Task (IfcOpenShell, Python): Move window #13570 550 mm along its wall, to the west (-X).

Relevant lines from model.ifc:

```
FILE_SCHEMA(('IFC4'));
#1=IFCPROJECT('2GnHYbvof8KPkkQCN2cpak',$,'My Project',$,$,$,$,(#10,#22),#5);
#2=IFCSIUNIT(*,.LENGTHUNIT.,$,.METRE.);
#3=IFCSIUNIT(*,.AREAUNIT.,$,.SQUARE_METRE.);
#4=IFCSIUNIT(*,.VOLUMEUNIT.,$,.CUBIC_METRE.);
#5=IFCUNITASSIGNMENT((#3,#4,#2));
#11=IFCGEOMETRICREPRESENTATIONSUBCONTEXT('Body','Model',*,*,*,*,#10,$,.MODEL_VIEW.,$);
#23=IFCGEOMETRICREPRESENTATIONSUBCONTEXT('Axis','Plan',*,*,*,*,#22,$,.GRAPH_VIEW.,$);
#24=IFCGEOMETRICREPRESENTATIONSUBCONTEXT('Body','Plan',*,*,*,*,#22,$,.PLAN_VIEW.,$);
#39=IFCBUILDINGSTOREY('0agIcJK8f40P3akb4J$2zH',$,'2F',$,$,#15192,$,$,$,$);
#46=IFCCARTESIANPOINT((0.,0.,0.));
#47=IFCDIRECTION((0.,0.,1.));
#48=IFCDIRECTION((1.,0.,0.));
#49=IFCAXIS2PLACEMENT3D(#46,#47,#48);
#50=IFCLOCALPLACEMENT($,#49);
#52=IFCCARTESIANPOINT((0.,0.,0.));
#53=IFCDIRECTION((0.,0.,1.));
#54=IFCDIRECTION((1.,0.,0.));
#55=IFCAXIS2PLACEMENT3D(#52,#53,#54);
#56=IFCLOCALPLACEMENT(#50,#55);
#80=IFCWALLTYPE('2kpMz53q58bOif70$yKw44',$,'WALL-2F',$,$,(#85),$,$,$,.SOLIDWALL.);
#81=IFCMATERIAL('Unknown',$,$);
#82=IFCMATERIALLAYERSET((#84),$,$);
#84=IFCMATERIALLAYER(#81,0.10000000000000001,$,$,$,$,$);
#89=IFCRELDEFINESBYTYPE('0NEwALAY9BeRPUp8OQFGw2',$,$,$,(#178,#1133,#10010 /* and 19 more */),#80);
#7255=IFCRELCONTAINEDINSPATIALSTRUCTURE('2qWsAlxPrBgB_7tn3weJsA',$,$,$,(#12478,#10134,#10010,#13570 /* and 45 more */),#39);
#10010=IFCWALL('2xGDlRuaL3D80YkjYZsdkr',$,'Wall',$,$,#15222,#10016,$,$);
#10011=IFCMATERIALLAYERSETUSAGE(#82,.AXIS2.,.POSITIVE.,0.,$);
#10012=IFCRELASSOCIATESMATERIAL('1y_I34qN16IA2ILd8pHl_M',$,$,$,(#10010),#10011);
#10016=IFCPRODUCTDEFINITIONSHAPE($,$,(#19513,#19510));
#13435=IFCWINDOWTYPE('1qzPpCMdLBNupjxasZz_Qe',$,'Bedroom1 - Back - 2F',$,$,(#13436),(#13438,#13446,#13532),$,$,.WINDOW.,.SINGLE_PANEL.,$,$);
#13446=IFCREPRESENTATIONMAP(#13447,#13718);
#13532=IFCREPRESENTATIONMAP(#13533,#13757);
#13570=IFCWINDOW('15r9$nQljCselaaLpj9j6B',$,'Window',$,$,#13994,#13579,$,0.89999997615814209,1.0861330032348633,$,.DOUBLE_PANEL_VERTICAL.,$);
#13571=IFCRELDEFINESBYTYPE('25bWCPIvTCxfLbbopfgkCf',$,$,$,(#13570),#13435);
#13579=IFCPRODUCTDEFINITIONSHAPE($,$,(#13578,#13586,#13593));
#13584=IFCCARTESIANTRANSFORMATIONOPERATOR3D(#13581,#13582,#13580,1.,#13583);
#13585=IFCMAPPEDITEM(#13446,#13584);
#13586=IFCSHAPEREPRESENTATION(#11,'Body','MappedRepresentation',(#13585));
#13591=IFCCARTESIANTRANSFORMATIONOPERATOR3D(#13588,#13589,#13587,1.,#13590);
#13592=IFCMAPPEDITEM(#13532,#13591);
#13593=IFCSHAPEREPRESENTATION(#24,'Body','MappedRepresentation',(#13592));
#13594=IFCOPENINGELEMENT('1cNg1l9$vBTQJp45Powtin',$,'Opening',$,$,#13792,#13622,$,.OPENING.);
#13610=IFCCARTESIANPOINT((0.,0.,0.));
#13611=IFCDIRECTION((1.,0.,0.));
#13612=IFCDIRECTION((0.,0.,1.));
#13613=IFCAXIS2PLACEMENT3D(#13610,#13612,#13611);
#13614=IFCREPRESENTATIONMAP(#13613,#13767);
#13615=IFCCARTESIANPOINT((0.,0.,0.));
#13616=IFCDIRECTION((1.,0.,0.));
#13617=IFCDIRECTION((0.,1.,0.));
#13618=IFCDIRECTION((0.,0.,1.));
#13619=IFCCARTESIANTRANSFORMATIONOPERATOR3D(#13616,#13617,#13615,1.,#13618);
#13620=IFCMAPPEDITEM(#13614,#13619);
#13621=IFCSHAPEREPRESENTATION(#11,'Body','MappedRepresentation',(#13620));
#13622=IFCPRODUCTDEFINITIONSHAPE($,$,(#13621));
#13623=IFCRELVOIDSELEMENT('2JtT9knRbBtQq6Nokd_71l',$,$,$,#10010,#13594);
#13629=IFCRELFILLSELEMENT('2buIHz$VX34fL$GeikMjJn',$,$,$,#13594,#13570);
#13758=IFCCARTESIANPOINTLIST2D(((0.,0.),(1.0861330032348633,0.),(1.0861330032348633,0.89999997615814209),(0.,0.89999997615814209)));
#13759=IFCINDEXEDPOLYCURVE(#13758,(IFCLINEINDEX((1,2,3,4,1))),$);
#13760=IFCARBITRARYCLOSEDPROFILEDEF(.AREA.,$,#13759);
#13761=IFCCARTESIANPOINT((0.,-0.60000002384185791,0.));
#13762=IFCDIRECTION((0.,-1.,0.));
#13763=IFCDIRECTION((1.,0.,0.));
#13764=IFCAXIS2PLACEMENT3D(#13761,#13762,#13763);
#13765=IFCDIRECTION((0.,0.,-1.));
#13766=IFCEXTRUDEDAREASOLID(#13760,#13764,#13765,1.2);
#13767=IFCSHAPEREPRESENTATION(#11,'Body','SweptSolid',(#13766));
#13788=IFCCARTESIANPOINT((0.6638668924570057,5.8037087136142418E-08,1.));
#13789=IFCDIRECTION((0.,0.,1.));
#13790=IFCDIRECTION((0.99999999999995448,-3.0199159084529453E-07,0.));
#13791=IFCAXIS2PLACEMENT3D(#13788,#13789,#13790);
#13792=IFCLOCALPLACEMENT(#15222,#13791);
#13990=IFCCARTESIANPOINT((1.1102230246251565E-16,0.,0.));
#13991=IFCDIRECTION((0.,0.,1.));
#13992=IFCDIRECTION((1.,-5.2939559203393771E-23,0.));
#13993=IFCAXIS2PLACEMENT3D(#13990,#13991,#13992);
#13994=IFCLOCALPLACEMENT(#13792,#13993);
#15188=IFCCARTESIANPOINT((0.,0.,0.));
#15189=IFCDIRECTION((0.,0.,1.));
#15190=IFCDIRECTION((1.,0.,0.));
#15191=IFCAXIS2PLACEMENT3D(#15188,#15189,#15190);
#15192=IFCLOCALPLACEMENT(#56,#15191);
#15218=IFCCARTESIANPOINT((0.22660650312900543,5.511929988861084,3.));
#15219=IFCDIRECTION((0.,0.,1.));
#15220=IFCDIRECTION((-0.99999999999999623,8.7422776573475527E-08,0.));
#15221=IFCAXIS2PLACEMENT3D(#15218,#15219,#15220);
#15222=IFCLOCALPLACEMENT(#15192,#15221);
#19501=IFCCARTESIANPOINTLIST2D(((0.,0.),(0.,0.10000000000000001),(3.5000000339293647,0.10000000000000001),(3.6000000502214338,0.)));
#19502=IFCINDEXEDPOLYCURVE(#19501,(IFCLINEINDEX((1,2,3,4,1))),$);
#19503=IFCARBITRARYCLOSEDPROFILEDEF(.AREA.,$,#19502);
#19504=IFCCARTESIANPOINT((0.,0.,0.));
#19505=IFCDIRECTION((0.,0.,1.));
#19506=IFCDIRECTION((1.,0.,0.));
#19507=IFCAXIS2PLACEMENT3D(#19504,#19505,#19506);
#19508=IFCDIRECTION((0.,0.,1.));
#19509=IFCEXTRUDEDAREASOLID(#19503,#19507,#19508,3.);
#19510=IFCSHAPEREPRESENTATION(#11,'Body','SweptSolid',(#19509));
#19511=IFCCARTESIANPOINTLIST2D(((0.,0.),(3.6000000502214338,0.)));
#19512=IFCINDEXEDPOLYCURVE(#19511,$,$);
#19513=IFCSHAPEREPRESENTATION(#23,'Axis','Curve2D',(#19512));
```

```python
import ifcopenshell
import ifcopenshell.api.geometry
import ifcopenshell.util.placement
import ifcopenshell.util.unit

model = ifcopenshell.open("model.ifc")
unit_scale = ifcopenshell.util.unit.calculate_unit_scale(model)

window = model.by_guid("15r9$nQljCselaaLpj9j6B")
opening = window.FillsVoids[0].RelatingOpeningElement
wall = opening.VoidsElements[0].RelatingBuildingElement

wall_matrix = ifcopenshell.util.placement.get_local_placement(wall.ObjectPlacement)
shift = wall_matrix[:3, 0] * 0.55 / unit_scale
before = ifcopenshell.util.placement.get_local_placement(window.ObjectPlacement)[:3, 3].copy()

# The window is placed relative to its opening, so it follows when the opening moves.
matrix = ifcopenshell.util.placement.get_local_placement(opening.ObjectPlacement)
matrix[:3, 3] += shift
ifcopenshell.api.geometry.edit_object_placement(
    model, product=opening, matrix=matrix, is_si=False, should_transform_children=True
)

after = ifcopenshell.util.placement.get_local_placement(window.ObjectPlacement)[:3, 3]
print("window moved by", (after - before).round(3) + 0.0)

model.write("model_updated.ifc")
```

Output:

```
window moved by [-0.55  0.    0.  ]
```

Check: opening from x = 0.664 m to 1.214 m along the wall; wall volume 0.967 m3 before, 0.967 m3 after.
